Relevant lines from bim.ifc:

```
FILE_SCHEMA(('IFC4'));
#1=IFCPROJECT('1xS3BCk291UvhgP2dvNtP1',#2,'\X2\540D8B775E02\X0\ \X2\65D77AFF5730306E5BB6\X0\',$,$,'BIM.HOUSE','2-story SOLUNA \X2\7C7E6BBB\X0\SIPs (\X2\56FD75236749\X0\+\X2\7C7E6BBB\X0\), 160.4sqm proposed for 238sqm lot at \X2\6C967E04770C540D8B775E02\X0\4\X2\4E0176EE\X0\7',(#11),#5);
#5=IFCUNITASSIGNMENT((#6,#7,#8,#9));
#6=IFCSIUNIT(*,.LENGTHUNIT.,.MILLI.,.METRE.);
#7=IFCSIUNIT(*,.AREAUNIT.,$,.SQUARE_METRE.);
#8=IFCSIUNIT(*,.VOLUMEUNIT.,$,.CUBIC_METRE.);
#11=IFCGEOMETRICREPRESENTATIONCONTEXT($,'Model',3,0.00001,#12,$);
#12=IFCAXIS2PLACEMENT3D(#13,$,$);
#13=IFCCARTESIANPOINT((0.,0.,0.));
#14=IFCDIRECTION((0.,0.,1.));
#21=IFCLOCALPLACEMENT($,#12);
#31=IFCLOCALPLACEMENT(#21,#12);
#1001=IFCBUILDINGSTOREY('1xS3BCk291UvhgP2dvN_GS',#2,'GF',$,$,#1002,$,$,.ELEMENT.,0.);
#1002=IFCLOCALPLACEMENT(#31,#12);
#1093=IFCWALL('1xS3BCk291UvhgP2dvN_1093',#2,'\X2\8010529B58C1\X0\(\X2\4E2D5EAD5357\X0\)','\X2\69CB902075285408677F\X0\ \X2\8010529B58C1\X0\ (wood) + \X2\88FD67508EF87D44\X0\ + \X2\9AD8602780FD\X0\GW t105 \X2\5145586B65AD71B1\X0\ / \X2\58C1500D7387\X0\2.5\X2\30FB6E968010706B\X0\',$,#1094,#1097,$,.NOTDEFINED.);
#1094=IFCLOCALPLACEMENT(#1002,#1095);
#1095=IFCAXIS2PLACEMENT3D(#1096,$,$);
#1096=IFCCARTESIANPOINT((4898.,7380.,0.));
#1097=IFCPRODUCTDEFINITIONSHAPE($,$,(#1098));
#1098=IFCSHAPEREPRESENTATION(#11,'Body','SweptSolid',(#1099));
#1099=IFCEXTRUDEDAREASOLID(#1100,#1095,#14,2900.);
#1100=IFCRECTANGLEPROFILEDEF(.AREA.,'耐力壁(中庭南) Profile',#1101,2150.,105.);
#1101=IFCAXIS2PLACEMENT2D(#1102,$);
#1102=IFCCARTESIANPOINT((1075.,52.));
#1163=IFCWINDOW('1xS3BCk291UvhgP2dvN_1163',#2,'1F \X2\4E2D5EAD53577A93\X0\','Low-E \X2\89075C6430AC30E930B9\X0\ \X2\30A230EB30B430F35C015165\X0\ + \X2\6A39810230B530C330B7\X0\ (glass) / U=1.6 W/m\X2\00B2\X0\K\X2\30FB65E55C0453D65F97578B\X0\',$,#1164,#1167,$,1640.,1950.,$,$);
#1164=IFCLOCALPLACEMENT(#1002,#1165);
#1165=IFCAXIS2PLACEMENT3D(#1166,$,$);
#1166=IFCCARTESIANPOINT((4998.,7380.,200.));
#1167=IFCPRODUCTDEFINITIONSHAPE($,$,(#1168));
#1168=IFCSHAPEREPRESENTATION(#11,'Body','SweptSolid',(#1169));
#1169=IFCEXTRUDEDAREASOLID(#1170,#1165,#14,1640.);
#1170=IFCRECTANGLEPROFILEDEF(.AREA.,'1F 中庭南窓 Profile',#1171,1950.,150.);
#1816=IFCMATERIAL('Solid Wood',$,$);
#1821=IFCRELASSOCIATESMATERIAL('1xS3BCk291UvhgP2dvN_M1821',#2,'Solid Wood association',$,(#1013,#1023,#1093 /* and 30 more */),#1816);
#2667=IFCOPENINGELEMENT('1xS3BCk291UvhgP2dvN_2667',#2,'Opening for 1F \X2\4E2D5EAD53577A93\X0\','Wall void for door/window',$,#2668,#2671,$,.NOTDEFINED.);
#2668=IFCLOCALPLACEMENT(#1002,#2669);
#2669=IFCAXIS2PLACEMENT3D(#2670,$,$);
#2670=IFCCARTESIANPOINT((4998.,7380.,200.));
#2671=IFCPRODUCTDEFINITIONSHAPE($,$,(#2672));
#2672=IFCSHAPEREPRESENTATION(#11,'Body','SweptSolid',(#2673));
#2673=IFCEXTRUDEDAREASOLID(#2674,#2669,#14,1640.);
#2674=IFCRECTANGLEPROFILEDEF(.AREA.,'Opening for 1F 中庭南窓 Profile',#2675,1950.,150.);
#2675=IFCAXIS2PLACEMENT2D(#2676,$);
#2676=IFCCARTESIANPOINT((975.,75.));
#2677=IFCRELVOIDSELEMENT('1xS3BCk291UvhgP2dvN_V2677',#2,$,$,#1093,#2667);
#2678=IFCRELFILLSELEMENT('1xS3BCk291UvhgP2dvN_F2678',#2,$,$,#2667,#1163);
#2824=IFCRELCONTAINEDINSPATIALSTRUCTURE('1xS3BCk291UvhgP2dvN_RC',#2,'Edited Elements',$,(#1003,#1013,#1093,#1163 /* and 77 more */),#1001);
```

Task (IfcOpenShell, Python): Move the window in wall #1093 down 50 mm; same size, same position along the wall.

```python
import numpy as np
import ifcopenshell
import ifcopenshell.api.geometry
import ifcopenshell.util.placement
import ifcopenshell.util.unit

model = ifcopenshell.open("bim.ifc")
unit_scale = ifcopenshell.util.unit.calculate_unit_scale(model)

window = model.by_id(1163)
opening = window.FillsVoids[0].RelatingOpeningElement
dz = -0.05 / unit_scale

shift = np.array([0.0, 0.0, dz])
# The window is not placed relative to its opening, so move both.
for product in (opening, window):
    matrix = ifcopenshell.util.placement.get_local_placement(product.ObjectPlacement)
    matrix[:3, 3] += shift
    ifcopenshell.api.geometry.edit_object_placement(model, product=product, matrix=matrix, is_si=False)

print(f"moved by {dz * unit_scale:+.3f} m")

model.write("bim_updated.ifc")
```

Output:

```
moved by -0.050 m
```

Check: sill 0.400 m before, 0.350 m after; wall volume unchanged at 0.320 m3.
